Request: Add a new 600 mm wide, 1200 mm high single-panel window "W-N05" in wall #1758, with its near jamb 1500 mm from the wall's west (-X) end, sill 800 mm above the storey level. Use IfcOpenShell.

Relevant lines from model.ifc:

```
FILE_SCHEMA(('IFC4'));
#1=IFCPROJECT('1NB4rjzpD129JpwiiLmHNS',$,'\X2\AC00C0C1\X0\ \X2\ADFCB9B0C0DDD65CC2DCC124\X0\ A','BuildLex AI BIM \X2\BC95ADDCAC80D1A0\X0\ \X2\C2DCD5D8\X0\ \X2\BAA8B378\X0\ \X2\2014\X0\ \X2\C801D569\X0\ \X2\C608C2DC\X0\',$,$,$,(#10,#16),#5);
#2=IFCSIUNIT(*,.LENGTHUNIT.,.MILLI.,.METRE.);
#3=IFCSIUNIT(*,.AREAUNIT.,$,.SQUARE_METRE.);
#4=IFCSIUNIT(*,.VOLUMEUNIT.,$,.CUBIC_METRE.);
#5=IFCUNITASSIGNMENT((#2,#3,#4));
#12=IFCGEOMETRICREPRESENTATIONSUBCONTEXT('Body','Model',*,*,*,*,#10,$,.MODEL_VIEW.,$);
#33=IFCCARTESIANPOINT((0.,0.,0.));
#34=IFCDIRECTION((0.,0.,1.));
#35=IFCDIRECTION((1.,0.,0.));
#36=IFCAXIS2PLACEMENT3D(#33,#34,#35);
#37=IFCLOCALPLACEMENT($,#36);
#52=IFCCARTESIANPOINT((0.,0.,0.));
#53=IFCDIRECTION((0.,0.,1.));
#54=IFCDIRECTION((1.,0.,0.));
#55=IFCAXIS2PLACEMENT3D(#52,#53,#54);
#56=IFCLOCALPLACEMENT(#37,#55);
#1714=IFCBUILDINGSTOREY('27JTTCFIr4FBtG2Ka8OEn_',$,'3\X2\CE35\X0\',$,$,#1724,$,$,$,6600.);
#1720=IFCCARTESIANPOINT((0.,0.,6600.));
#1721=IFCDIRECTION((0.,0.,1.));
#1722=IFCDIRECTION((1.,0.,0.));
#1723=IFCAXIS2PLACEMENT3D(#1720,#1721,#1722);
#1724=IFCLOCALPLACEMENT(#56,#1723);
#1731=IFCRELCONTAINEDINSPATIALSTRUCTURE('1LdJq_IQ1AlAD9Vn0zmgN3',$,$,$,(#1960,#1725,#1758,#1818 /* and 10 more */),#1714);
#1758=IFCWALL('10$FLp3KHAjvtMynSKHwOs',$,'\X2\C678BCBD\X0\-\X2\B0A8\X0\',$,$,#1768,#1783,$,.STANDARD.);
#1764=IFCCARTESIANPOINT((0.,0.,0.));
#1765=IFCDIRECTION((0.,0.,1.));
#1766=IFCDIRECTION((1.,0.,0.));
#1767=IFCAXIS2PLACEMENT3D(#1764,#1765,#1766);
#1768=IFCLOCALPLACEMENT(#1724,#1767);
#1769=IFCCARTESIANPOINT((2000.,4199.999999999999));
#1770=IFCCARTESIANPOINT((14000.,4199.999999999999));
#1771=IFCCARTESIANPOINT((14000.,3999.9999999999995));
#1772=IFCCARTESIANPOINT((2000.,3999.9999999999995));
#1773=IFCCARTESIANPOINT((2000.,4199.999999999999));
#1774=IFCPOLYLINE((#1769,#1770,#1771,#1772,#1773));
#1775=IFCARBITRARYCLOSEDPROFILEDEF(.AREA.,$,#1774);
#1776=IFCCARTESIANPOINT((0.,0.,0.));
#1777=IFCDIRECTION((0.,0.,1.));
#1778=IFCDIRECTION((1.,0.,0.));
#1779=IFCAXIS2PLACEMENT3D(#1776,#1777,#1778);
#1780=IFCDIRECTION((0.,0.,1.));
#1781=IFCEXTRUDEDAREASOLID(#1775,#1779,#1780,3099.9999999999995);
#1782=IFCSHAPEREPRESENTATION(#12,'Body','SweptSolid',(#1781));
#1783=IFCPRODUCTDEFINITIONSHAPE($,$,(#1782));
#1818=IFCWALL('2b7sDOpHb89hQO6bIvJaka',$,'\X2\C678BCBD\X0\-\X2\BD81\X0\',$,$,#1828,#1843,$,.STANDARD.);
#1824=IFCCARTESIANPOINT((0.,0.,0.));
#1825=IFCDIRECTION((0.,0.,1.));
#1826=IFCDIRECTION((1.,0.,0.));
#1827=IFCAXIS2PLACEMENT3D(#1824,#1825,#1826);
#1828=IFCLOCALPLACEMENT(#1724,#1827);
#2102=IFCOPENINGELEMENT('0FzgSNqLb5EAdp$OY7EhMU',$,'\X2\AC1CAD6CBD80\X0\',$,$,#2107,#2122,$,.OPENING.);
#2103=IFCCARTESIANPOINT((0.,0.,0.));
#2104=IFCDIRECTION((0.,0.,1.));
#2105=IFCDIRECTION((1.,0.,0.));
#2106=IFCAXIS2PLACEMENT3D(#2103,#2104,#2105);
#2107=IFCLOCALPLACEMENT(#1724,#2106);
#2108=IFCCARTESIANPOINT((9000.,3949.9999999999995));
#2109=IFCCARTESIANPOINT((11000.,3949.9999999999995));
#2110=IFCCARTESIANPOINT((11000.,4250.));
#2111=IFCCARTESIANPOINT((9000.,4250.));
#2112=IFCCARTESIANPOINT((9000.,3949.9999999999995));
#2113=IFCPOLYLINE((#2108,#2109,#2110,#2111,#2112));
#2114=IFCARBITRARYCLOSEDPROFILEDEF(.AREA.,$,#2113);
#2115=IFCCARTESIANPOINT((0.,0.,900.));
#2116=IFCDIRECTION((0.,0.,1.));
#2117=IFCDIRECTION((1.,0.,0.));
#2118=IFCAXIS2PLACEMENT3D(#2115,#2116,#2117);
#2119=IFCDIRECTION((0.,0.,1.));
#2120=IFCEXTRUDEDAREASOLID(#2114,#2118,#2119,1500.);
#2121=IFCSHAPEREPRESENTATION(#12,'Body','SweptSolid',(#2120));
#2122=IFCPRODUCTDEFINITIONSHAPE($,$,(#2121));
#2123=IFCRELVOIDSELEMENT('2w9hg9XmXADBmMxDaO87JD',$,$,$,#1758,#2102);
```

```python
import numpy as np
import ifcopenshell
import ifcopenshell.api.feature
import ifcopenshell.api.geometry
import ifcopenshell.api.root
import ifcopenshell.api.spatial
import ifcopenshell.geom
import ifcopenshell.util.element
import ifcopenshell.util.placement
import ifcopenshell.util.representation
import ifcopenshell.util.shape
import ifcopenshell.util.unit

model = ifcopenshell.open("model.ifc")
unit_scale = ifcopenshell.util.unit.calculate_unit_scale(model)
settings = ifcopenshell.geom.settings()


def volume(element):
    """Net volume in cubic metres, openings subtracted."""
    shape = ifcopenshell.geom.create_shape(settings, element)
    return ifcopenshell.util.shape.get_volume(shape.geometry)


wall = model.by_guid("10$FLp3KHAjvtMynSKHwOs")
storey = ifcopenshell.util.element.get_container(wall, ifc_class="IfcBuildingStorey")
context = ifcopenshell.util.representation.get_context(model, "Model", "Body", "MODEL_VIEW")
before = volume(wall)

width, height, from_end, sill = 0.6, 1.2, 1.5, 0.8  # metres

# The wall runs along its own X axis, and the end named is its -X end.
wall_shape = ifcopenshell.geom.create_shape(settings, wall)
x, y, z = ifcopenshell.util.shape.get_vertices(wall_shape.geometry).T
start = x.min() + from_end
face, thickness = float(y.min()), float(y.max() - y.min())
wall_matrix = ifcopenshell.util.placement.get_local_placement(wall.ObjectPlacement)
level = ifcopenshell.util.placement.get_local_placement(storey.ObjectPlacement)[2, 3]


def in_wall(x, y):
    """Placement at x, y metres in the wall's axes, at sill height."""
    matrix = wall_matrix.copy()
    matrix[:, 3] = wall_matrix @ np.array([x / unit_scale, y / unit_scale, 0.0, 1.0])
    matrix[2, 3] = level + sill / unit_scale
    return matrix


# Opening: a box that overshoots both wall faces by 50 mm.
opening = ifcopenshell.api.root.create_entity(model, ifc_class="IfcOpeningElement", predefined_type="OPENING")
box = ifcopenshell.api.geometry.add_wall_representation(
    model, context=context, length=width, height=height, thickness=thickness + 0.1
)
ifcopenshell.api.geometry.assign_representation(model, product=opening, representation=box)
ifcopenshell.api.geometry.edit_object_placement(model, product=opening, matrix=in_wall(start, face - 0.05), is_si=False)
ifcopenshell.api.feature.add_feature(model, feature=opening, element=wall)

window = ifcopenshell.api.root.create_entity(model, ifc_class="IfcWindow", name="W-N05", predefined_type="WINDOW")
window.OverallWidth, window.OverallHeight = width / unit_scale, height / unit_scale
window.PartitioningType = "SINGLE_PANEL"
body = ifcopenshell.api.geometry.add_window_representation(
    model,
    context=context,
    overall_width=window.OverallWidth,
    overall_height=window.OverallHeight,
    partition_type="SINGLE_PANEL",
)
ifcopenshell.api.geometry.assign_representation(model, product=window, representation=body)
ifcopenshell.api.spatial.assign_container(model, products=[window], relating_structure=storey)
ifcopenshell.api.feature.add_filling(model, opening=opening, element=window)

# Centre the window in the wall's thickness.
ifcopenshell.api.geometry.edit_object_placement(model, product=window, matrix=in_wall(start, face), is_si=False)
window_shape = ifcopenshell.geom.create_shape(settings, window)
depth = ifcopenshell.util.shape.get_vertices(window_shape.geometry)[:, 1]
offset = face + thickness / 2 - (depth.min() + depth.max()) / 2
ifcopenshell.api.geometry.edit_object_placement(model, product=window, matrix=in_wall(start, offset), is_si=False)

after = volume(wall)

print(f"wall volume {before:.3f} -> {after:.3f} m3")

model.write("model_v2.ifc")
```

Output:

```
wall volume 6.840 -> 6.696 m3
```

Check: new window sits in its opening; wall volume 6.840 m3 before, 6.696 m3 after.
